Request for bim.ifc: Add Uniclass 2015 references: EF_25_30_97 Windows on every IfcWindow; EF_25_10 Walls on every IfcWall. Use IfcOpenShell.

First a look at what the model holds.

```python
import ifcopenshell

model = ifcopenshell.open("bim.ifc")
print(model.schema)
print("classifications:", [c.Name for c in model.by_type("IfcClassification")])
for ifc_class in ("IfcDoor", "IfcRoof", "IfcStair", "IfcWall", "IfcWindow"):
    print(ifc_class, len(model.by_type(ifc_class)))
```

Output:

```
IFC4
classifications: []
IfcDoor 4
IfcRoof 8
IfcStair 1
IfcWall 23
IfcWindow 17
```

```python
import ifcopenshell
import ifcopenshell.api.classification

model = ifcopenshell.open("bim.ifc")

system = ifcopenshell.api.classification.add_classification(model, classification="Uniclass 2015")

codes = {
    "IfcWindow": ("EF_25_30_97", "Windows"),
    "IfcWall": ("EF_25_10", "Walls"),
}
for ifc_class, (code, name) in codes.items():
    products = model.by_type(ifc_class)
    ifcopenshell.api.classification.add_reference(
        model, products=products, classification=system, identification=code, name=name
    )
    print(code, len(products))

model.write("bim-out.ifc")
```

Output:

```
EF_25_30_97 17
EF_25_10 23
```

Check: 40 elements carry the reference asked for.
